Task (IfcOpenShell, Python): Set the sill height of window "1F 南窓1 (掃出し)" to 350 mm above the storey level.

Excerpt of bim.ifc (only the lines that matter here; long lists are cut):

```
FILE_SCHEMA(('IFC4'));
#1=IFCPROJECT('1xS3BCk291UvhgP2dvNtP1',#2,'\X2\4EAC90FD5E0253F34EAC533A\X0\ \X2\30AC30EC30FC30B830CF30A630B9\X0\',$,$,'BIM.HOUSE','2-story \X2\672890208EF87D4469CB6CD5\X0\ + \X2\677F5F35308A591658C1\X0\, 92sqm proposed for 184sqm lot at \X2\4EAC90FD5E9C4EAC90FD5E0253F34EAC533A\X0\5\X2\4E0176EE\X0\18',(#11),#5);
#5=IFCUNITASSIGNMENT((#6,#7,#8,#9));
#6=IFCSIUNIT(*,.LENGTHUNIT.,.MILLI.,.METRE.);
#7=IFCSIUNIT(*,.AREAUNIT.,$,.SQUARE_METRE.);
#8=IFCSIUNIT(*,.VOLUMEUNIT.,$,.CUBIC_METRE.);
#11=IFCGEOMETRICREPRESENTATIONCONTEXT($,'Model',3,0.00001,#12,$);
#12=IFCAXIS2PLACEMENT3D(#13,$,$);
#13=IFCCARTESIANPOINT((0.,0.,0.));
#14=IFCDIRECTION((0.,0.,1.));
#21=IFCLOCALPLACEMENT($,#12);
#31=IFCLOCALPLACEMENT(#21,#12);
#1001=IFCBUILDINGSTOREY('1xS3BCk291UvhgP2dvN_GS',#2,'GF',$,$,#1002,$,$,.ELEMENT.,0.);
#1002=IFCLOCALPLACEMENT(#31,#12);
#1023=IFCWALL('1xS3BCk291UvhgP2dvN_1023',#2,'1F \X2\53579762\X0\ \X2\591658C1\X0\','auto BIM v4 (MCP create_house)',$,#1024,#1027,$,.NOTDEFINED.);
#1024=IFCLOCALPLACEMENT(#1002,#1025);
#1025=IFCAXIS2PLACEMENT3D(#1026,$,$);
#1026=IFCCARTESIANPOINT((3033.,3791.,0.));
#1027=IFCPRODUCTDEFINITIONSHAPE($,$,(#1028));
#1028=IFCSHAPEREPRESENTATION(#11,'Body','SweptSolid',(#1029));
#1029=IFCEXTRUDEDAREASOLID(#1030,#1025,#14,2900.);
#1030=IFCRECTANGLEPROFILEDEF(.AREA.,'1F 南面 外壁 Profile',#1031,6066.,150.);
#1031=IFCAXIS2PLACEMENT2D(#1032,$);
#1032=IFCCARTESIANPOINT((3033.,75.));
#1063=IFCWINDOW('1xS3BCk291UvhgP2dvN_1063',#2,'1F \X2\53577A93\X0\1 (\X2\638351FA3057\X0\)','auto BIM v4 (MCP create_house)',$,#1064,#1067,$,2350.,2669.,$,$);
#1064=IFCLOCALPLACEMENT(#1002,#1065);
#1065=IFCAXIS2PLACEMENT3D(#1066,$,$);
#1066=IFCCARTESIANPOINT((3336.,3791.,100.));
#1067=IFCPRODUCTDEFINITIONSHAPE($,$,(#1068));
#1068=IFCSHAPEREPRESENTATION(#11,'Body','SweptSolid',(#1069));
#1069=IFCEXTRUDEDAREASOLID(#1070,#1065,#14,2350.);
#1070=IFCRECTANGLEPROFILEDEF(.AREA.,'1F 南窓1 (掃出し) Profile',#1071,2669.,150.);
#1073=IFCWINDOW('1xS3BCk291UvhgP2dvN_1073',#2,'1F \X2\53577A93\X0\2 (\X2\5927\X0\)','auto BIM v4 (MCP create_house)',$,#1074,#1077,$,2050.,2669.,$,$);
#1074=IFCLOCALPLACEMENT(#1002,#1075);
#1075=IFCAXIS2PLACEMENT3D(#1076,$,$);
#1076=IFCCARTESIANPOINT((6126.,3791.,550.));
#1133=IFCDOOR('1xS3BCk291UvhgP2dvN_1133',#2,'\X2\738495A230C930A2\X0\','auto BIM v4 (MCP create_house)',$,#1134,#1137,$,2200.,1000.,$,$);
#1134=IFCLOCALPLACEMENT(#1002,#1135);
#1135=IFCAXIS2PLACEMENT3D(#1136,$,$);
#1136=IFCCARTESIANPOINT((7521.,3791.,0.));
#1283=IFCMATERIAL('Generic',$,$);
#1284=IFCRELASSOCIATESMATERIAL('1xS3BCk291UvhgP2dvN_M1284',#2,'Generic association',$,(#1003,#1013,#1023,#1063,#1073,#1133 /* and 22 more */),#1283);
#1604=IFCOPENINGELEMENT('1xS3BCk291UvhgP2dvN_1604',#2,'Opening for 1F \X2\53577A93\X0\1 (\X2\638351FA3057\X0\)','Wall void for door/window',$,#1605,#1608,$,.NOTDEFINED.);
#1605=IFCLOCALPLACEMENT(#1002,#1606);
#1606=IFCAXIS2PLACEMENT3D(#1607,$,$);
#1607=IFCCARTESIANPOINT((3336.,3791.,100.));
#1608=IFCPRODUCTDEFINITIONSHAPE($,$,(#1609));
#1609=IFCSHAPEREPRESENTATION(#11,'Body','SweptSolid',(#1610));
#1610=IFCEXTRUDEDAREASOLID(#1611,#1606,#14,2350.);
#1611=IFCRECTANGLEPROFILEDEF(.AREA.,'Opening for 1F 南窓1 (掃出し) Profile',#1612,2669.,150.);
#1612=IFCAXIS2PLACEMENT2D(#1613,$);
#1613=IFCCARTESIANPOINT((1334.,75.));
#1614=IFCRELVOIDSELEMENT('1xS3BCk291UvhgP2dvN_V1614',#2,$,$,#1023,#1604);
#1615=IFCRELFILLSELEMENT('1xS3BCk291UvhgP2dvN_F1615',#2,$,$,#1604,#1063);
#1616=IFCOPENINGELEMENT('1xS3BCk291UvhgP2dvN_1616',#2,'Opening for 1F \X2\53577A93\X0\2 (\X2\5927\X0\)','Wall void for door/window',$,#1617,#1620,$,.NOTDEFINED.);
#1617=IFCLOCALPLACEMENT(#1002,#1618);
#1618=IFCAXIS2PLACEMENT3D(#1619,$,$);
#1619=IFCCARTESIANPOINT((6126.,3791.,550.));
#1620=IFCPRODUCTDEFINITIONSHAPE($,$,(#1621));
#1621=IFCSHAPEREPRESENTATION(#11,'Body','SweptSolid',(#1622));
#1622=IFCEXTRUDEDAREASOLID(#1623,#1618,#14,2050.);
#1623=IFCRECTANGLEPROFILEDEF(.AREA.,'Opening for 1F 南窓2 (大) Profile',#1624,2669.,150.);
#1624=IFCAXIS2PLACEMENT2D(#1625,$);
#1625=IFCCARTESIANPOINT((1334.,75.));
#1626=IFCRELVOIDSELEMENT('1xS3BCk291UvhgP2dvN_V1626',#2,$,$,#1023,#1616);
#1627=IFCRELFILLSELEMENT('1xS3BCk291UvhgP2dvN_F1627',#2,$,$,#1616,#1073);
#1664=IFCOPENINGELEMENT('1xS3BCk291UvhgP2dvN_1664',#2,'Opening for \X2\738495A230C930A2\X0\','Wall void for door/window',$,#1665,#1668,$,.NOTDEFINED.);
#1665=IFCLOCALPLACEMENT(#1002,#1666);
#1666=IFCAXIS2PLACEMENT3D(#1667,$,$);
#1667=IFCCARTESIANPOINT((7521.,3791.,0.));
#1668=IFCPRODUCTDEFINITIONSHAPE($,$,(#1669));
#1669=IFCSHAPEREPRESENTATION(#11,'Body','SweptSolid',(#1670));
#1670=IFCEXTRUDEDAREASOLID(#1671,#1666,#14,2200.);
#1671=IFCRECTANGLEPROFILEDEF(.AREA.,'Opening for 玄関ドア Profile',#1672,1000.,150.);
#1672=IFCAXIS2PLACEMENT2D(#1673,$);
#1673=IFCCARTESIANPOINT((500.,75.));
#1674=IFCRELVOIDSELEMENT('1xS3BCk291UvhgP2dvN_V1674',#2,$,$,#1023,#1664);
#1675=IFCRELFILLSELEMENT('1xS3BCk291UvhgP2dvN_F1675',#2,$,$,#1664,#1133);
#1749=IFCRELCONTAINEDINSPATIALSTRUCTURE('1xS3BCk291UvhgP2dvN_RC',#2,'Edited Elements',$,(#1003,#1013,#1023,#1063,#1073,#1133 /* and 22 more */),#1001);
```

```python
import numpy as np
import ifcopenshell
import ifcopenshell.api.geometry
import ifcopenshell.geom
import ifcopenshell.util.element
import ifcopenshell.util.placement
import ifcopenshell.util.shape
import ifcopenshell.util.unit

model = ifcopenshell.open("bim.ifc")
unit_scale = ifcopenshell.util.unit.calculate_unit_scale(model)

window = model.by_guid("1xS3BCk291UvhgP2dvN_1063")
opening = window.FillsVoids[0].RelatingOpeningElement
storey = ifcopenshell.util.element.get_container(window, ifc_class="IfcBuildingStorey")
level = ifcopenshell.util.placement.get_local_placement(storey.ObjectPlacement)[2, 3]

# The opening's origin need not be at the sill, so measure its lowest point.
shape = ifcopenshell.geom.create_shape(ifcopenshell.geom.settings(), opening)
bottom = ifcopenshell.util.shape.get_shape_bottom_elevation(shape, shape.geometry) / unit_scale
dz = level + 350.0 - bottom

shift = np.array([0.0, 0.0, dz])
# The window is not placed relative to its opening, so move both.
for product in (opening, window):
    matrix = ifcopenshell.util.placement.get_local_placement(product.ObjectPlacement)
    matrix[:3, 3] += shift
    ifcopenshell.api.geometry.edit_object_placement(model, product=product, matrix=matrix, is_si=False)

print(f"moved by {dz * unit_scale:+.3f} m")

model.write("bim_updated.ifc")
```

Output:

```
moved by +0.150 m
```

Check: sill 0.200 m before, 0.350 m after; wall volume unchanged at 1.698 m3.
